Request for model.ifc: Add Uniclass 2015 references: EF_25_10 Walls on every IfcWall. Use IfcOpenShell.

First a look at what the model holds.

```python
import ifcopenshell

model = ifcopenshell.open("model.ifc")
print(model.schema)
print("classifications:", [c.Name for c in model.by_type("IfcClassification")])
for ifc_class in ("IfcDoor", "IfcRoof", "IfcStair", "IfcWall", "IfcWindow"):
    print(ifc_class, len(model.by_type(ifc_class)))
```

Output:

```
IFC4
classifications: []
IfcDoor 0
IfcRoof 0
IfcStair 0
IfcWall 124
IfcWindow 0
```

```python
import ifcopenshell
import ifcopenshell.api.classification

model = ifcopenshell.open("model.ifc")

system = ifcopenshell.api.classification.add_classification(model, classification="Uniclass 2015")

codes = {
    "IfcWall": ("EF_25_10", "Walls"),
}
for ifc_class, (code, name) in codes.items():
    products = model.by_type(ifc_class)
    ifcopenshell.api.classification.add_reference(
        model, products=products, classification=system, identification=code, name=name
    )
    print(code, len(products))

model.write("model_v2.ifc")
```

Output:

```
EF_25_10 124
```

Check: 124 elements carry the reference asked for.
